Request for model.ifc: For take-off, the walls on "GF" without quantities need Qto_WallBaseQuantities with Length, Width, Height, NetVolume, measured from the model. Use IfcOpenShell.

First a look at what the model holds.

```python
import ifcopenshell
import ifcopenshell.util.element
import ifcopenshell.util.unit

model = ifcopenshell.open("model.ifc")
print(model.schema)
for unit_type in ("LENGTHUNIT", "AREAUNIT", "VOLUMEUNIT"):
    print(unit_type, ifcopenshell.util.unit.calculate_unit_scale(model, unit_type))
storey = next(s for s in model.by_type("IfcBuildingStorey") if s.Name == "GF")
walls = [e for e in ifcopenshell.util.element.get_decomposition(storey) if e.is_a("IfcWall")]
for e in sorted(walls, key=lambda e: e.id()):
    print(e.id(), e.is_a(), e.Name, list(ifcopenshell.util.element.get_psets(e, qtos_only=True)), sep=" | ")
```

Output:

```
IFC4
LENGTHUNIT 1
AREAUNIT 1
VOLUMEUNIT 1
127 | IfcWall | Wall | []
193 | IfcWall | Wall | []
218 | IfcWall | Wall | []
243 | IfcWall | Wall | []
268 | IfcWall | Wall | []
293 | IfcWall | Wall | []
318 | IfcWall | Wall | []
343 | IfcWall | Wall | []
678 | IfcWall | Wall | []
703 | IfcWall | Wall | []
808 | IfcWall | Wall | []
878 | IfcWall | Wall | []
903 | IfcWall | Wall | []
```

```python
import ifcopenshell
import ifcopenshell.api.pset
import ifcopenshell.geom
import ifcopenshell.util.element
import ifcopenshell.util.shape
import ifcopenshell.util.unit

model = ifcopenshell.open("model.ifc")
unit_scale = ifcopenshell.util.unit.calculate_unit_scale(model)
volume_scale = ifcopenshell.util.unit.calculate_unit_scale(model, "VOLUMEUNIT")
settings = ifcopenshell.geom.settings()

storey = next(s for s in model.by_type("IfcBuildingStorey") if s.Name == "GF")
walls = [e for e in ifcopenshell.util.element.get_decomposition(storey) if e.is_a("IfcWall")]

for e in sorted(walls, key=lambda e: e.id()):
    if ifcopenshell.util.element.get_psets(e, qtos_only=True, should_inherit=False):
        continue
    # Geometry comes back in metres, in the element's own axes.
    shape = ifcopenshell.geom.create_shape(settings, e)
    values = {
        "Length": ifcopenshell.util.shape.get_x(shape.geometry) / unit_scale,
        "Width": ifcopenshell.util.shape.get_y(shape.geometry) / unit_scale,
        "Height": ifcopenshell.util.shape.get_z(shape.geometry) / unit_scale,
        "NetVolume": ifcopenshell.util.shape.get_volume(shape.geometry) / volume_scale,
    }
    qto = ifcopenshell.api.pset.add_qto(model, product=e, name="Qto_WallBaseQuantities")
    ifcopenshell.api.pset.edit_qto(model, qto=qto, properties=values)
    print(e.id(), {k: round(v, 3) for k, v in values.items()})

model.write("model-out.ifc")
```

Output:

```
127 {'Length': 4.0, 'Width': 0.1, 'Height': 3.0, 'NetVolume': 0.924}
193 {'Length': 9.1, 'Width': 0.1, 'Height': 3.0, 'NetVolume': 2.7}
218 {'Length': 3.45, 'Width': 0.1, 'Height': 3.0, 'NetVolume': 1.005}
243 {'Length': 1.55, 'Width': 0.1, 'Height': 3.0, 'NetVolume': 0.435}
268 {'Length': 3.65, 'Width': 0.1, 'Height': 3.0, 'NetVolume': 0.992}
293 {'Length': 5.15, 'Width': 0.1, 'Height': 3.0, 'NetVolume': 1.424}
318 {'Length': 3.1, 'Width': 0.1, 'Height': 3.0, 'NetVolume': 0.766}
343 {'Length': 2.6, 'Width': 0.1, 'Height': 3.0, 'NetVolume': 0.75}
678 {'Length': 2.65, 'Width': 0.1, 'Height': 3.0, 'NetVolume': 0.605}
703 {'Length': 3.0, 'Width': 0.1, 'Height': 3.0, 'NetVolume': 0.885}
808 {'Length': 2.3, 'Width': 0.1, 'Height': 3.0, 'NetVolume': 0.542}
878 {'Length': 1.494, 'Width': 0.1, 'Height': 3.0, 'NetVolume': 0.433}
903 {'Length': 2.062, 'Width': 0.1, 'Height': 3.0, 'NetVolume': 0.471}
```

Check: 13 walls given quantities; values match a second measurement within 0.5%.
